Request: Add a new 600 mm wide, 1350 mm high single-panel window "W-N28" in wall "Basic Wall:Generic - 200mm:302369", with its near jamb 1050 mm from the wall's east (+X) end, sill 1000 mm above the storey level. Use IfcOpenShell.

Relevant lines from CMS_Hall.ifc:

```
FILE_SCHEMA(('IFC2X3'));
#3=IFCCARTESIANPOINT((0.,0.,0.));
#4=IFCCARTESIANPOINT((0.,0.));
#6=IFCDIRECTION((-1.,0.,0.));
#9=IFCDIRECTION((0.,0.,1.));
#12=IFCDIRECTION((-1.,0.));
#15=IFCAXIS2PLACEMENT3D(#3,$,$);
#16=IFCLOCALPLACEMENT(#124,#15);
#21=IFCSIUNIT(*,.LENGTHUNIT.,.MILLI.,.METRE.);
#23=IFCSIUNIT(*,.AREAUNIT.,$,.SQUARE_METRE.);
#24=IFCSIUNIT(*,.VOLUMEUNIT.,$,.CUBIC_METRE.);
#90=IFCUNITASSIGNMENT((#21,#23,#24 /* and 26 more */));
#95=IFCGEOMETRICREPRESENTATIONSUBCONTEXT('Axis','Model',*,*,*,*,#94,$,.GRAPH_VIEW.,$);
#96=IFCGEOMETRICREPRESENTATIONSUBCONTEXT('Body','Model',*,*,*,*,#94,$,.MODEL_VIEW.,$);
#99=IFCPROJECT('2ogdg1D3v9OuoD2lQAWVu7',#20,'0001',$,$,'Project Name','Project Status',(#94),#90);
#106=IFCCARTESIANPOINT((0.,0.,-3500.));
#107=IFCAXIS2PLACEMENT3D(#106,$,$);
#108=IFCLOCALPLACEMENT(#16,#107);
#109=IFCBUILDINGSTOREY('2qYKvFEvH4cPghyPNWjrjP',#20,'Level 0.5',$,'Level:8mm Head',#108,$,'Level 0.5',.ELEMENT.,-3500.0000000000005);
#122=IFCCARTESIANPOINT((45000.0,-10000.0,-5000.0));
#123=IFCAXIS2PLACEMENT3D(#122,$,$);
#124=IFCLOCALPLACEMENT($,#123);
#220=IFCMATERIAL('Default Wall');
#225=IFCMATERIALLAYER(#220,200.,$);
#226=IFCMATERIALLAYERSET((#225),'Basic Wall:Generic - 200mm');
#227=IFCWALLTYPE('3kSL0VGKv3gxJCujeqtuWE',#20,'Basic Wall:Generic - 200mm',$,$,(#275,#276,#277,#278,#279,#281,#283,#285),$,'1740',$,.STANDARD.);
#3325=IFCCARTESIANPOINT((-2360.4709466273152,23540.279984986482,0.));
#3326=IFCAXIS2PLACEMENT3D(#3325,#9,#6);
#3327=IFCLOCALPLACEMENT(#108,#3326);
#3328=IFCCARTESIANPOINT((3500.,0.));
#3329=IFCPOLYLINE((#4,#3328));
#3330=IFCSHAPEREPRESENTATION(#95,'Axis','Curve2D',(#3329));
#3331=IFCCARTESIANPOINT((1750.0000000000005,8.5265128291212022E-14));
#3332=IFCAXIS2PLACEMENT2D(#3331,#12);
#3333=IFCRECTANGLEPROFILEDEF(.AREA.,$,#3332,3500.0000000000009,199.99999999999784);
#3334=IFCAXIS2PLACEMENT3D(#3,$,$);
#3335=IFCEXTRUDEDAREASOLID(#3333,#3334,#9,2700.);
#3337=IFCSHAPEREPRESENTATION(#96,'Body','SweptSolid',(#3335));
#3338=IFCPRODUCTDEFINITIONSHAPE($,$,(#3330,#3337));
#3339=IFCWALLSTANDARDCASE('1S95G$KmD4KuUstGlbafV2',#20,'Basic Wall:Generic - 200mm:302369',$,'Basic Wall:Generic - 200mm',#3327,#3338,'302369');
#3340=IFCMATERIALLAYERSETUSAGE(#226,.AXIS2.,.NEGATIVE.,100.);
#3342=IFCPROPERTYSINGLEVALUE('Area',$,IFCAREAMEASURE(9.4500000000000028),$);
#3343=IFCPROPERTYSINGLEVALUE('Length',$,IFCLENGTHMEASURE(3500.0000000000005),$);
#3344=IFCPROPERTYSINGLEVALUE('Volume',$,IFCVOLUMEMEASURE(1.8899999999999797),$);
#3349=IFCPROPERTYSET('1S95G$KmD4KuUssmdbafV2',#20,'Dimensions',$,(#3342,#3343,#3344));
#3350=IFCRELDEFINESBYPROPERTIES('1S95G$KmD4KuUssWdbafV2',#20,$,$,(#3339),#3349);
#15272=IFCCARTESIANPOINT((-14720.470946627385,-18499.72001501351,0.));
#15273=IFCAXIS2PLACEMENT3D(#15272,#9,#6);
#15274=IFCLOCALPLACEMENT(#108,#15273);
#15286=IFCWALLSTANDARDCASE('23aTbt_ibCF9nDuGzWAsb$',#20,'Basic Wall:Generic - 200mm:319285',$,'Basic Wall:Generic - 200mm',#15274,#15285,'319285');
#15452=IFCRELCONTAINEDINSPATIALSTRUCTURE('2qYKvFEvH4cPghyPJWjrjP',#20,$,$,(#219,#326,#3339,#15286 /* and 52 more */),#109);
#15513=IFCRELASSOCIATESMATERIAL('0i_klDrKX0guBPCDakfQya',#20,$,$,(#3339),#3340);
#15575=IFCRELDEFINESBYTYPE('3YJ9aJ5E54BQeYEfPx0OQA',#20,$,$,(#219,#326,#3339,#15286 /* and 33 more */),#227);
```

```python
import numpy as np
import ifcopenshell
import ifcopenshell.api.feature
import ifcopenshell.api.geometry
import ifcopenshell.api.pset
import ifcopenshell.api.root
import ifcopenshell.api.spatial
import ifcopenshell.api.type
import ifcopenshell.geom
import ifcopenshell.util.element
import ifcopenshell.util.placement
import ifcopenshell.util.representation
import ifcopenshell.util.shape
import ifcopenshell.util.unit

model = ifcopenshell.open("CMS_Hall.ifc")
unit_scale = ifcopenshell.util.unit.calculate_unit_scale(model)
area_scale = ifcopenshell.util.unit.calculate_unit_scale(model, "AREAUNIT")
volume_scale = ifcopenshell.util.unit.calculate_unit_scale(model, "VOLUMEUNIT")
settings = ifcopenshell.geom.settings()


def volume(element):
    """Net volume in cubic metres, openings subtracted."""
    shape = ifcopenshell.geom.create_shape(settings, element)
    return ifcopenshell.util.shape.get_volume(shape.geometry)


wall = model.by_id(3339)
storey = ifcopenshell.util.element.get_container(wall, ifc_class="IfcBuildingStorey")
context = ifcopenshell.util.representation.get_context(model, "Model", "Body", "MODEL_VIEW")
before = volume(wall)

width, height, from_end, sill = 0.6, 1.35, 1.05, 1  # metres

# The wall runs along its own X axis, and the end named is its -X end.
wall_shape = ifcopenshell.geom.create_shape(settings, wall)
x, y, z = ifcopenshell.util.shape.get_vertices(wall_shape.geometry).T
start = x.min() + from_end
face, thickness = float(y.min()), float(y.max() - y.min())
wall_matrix = ifcopenshell.util.placement.get_local_placement(wall.ObjectPlacement)
level = ifcopenshell.util.placement.get_local_placement(storey.ObjectPlacement)[2, 3]


def in_wall(x, y):
    """Placement at x, y metres in the wall's axes, at sill height."""
    matrix = wall_matrix.copy()
    matrix[:, 3] = wall_matrix @ np.array([x / unit_scale, y / unit_scale, 0.0, 1.0])
    matrix[2, 3] = level + sill / unit_scale
    return matrix


# Opening: a box that overshoots both wall faces by 50 mm.
opening = ifcopenshell.api.root.create_entity(model, ifc_class="IfcOpeningElement")
box = ifcopenshell.api.geometry.add_wall_representation(
    model, context=context, length=width, height=height, thickness=thickness + 0.1
)
ifcopenshell.api.geometry.assign_representation(model, product=opening, representation=box)
ifcopenshell.api.geometry.edit_object_placement(model, product=opening, matrix=in_wall(start, face - 0.05), is_si=False)
ifcopenshell.api.feature.add_feature(model, feature=opening, element=wall)

window = ifcopenshell.api.root.create_entity(model, ifc_class="IfcWindow", name="W-N28")
window.OverallWidth, window.OverallHeight = width / unit_scale, height / unit_scale
body = ifcopenshell.api.geometry.add_window_representation(
    model,
    context=context,
    overall_width=window.OverallWidth,
    overall_height=window.OverallHeight,
    partition_type="SINGLE_PANEL",
)
ifcopenshell.api.geometry.assign_representation(model, product=window, representation=body)
ifcopenshell.api.spatial.assign_container(model, products=[window], relating_structure=storey)
fills = ifcopenshell.api.feature.add_filling(model, opening=opening, element=window)
fills.OwnerHistory = window.OwnerHistory  # required in IFC2X3

# IFC2X3 keeps the operation on the window style.
style = ifcopenshell.api.root.create_entity(model, ifc_class="IfcWindowStyle", name="W-N28")
style.OperationType, style.ConstructionType = "SINGLE_PANEL", "NOTDEFINED"
style.ParameterTakesPrecedence = style.Sizeable = False
ifcopenshell.api.type.assign_type(model, related_objects=[window], relating_type=style)

# Centre the window in the wall's thickness.
ifcopenshell.api.geometry.edit_object_placement(model, product=window, matrix=in_wall(start, face), is_si=False)
window_shape = ifcopenshell.geom.create_shape(settings, window)
depth = ifcopenshell.util.shape.get_vertices(window_shape.geometry)[:, 1]
offset = face + thickness / 2 - (depth.min() + depth.max()) / 2
ifcopenshell.api.geometry.edit_object_placement(model, product=window, matrix=in_wall(start, offset), is_si=False)

after = volume(wall)

# Update the wall's stored quantities.
pset = model.by_id(ifcopenshell.util.element.get_pset(wall, "Dimensions", should_inherit=False)["id"])
ifcopenshell.api.pset.edit_pset(model, pset=pset, properties={
    "Area": model.create_entity("IfcAreaMeasure", after / thickness / area_scale),
    "Volume": model.create_entity("IfcVolumeMeasure", after / volume_scale),
})

print(f"wall volume {before:.3f} -> {after:.3f} m3")

model.write("CMS_Hall_rev.ifc")
```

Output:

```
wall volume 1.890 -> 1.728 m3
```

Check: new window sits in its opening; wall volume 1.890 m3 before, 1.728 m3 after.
